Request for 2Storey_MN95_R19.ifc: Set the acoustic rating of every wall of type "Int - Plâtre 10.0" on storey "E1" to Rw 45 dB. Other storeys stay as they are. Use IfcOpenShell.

First a look at what the model holds.

```python
import ifcopenshell
import ifcopenshell.util.element

model = ifcopenshell.open("2Storey_MN95_R19.ifc")
print(model.schema)
storey = next(s for s in model.by_type("IfcBuildingStorey") if s.Name == "E1")
walls = [e for e in ifcopenshell.util.element.get_decomposition(storey) if e.is_a("IfcWall")]
seen = {}
for e in walls:
    element_type = ifcopenshell.util.element.get_type(e)
    key = (element_type.Name if element_type != e and element_type else None, ifcopenshell.util.element.get_pset(e, "Pset_WallCommon", "AcousticRating"))
    seen[key] = seen.get(key, 0) + 1
for (name, value), count in sorted(seen.items(), key=str):
    print(count, "x", name, "|", value)
```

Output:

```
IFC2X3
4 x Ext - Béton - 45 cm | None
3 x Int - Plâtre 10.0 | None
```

```python
import ifcopenshell
import ifcopenshell.api.pset
import ifcopenshell.util.element

model = ifcopenshell.open("2Storey_MN95_R19.ifc")

storey = next(s for s in model.by_type("IfcBuildingStorey") if s.Name == "E1")
walls = [e for e in ifcopenshell.util.element.get_decomposition(storey) if e.is_a("IfcWall")]

count = 0
for e in walls:
    element_type = ifcopenshell.util.element.get_type(e)
    if element_type in (None, e) or element_type.Name != "Int - Plâtre 10.0":
        continue
    # add_pset returns the element's existing set when there is one.
    pset = ifcopenshell.api.pset.add_pset(model, product=e, name="Pset_WallCommon")
    ifcopenshell.api.pset.edit_pset(model, pset=pset, properties={"AcousticRating": "Rw 45 dB"})
    count += 1

print(count, "walls updated")

model.write("2Storey_MN95_R19_edited.ifc")
```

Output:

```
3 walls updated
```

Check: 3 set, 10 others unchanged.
